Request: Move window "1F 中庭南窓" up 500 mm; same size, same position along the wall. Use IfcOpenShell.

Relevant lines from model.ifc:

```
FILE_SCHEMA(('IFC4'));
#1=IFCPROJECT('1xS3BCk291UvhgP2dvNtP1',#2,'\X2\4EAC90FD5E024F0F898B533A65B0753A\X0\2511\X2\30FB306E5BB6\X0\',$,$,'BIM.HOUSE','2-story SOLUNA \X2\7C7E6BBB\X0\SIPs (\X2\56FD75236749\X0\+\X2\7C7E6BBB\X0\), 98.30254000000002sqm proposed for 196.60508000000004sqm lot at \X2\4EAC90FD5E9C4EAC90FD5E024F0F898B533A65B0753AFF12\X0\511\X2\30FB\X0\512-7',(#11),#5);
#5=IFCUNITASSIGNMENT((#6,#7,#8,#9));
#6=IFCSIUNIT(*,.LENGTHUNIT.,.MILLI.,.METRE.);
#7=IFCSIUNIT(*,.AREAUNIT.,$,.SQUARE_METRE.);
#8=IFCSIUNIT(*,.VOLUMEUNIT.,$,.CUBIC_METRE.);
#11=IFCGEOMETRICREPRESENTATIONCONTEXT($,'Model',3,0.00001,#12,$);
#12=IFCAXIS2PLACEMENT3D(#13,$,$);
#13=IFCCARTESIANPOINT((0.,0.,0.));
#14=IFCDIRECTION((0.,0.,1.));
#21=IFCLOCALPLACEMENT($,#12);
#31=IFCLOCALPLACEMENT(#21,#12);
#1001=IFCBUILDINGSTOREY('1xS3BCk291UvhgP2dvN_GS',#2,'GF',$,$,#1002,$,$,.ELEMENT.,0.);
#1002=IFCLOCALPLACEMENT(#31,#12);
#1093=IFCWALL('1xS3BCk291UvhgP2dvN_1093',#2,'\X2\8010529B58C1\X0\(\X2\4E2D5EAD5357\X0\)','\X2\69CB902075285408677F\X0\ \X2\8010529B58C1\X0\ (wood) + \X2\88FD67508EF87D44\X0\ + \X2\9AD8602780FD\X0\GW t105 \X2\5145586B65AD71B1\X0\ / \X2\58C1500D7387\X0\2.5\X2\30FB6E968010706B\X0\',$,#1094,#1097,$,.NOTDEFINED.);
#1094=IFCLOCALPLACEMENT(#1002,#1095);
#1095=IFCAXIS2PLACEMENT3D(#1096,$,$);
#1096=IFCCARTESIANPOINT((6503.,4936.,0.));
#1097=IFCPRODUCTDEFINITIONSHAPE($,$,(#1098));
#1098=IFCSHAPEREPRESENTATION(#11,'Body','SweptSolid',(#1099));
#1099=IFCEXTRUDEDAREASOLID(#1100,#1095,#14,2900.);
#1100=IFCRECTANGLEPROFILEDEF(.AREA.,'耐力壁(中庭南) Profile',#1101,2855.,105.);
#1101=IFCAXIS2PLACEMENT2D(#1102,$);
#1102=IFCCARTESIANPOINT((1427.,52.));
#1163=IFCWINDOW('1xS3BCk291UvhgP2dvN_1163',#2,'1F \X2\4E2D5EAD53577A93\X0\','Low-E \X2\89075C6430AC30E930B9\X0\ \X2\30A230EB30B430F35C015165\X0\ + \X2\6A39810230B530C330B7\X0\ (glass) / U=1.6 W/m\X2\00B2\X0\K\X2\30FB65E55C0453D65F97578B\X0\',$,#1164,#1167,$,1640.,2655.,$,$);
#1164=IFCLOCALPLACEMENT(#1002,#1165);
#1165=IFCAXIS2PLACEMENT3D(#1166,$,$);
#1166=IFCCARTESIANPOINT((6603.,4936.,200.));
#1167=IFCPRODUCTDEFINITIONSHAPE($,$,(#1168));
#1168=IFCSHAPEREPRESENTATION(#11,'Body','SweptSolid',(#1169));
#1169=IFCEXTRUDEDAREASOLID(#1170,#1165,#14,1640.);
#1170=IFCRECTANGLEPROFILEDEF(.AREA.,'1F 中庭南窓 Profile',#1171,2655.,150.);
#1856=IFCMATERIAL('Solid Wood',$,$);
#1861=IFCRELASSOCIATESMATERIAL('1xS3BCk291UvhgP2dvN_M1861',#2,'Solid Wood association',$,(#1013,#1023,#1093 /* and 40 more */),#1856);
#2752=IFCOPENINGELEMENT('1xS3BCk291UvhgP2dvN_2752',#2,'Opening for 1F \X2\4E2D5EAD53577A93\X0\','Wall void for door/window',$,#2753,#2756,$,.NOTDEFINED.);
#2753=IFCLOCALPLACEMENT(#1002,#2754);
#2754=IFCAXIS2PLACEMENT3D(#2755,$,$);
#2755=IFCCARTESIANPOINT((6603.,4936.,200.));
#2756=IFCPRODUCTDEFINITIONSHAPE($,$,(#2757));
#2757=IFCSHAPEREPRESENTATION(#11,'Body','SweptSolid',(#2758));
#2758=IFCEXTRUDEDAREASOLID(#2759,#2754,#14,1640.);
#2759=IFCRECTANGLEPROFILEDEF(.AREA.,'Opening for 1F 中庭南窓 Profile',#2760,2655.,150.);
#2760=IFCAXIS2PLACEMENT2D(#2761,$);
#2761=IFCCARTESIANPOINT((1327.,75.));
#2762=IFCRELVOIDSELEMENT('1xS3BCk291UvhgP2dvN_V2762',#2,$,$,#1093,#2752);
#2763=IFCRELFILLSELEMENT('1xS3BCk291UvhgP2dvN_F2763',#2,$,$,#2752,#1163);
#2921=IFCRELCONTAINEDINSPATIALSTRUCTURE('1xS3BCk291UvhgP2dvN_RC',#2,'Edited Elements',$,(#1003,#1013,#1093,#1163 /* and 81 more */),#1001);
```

```python
import numpy as np
import ifcopenshell
import ifcopenshell.api.geometry
import ifcopenshell.util.placement
import ifcopenshell.util.unit

model = ifcopenshell.open("model.ifc")
unit_scale = ifcopenshell.util.unit.calculate_unit_scale(model)

window = model.by_guid("1xS3BCk291UvhgP2dvN_1163")
opening = window.FillsVoids[0].RelatingOpeningElement
dz = 0.5 / unit_scale

shift = np.array([0.0, 0.0, dz])
# The window is not placed relative to its opening, so move both.
for product in (opening, window):
    matrix = ifcopenshell.util.placement.get_local_placement(product.ObjectPlacement)
    matrix[:3, 3] += shift
    ifcopenshell.api.geometry.edit_object_placement(model, product=product, matrix=matrix, is_si=False)

print(f"moved by {dz * unit_scale:+.3f} m")

model.write("model_edited.ifc")
```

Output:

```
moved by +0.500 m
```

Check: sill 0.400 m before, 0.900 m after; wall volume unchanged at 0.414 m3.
